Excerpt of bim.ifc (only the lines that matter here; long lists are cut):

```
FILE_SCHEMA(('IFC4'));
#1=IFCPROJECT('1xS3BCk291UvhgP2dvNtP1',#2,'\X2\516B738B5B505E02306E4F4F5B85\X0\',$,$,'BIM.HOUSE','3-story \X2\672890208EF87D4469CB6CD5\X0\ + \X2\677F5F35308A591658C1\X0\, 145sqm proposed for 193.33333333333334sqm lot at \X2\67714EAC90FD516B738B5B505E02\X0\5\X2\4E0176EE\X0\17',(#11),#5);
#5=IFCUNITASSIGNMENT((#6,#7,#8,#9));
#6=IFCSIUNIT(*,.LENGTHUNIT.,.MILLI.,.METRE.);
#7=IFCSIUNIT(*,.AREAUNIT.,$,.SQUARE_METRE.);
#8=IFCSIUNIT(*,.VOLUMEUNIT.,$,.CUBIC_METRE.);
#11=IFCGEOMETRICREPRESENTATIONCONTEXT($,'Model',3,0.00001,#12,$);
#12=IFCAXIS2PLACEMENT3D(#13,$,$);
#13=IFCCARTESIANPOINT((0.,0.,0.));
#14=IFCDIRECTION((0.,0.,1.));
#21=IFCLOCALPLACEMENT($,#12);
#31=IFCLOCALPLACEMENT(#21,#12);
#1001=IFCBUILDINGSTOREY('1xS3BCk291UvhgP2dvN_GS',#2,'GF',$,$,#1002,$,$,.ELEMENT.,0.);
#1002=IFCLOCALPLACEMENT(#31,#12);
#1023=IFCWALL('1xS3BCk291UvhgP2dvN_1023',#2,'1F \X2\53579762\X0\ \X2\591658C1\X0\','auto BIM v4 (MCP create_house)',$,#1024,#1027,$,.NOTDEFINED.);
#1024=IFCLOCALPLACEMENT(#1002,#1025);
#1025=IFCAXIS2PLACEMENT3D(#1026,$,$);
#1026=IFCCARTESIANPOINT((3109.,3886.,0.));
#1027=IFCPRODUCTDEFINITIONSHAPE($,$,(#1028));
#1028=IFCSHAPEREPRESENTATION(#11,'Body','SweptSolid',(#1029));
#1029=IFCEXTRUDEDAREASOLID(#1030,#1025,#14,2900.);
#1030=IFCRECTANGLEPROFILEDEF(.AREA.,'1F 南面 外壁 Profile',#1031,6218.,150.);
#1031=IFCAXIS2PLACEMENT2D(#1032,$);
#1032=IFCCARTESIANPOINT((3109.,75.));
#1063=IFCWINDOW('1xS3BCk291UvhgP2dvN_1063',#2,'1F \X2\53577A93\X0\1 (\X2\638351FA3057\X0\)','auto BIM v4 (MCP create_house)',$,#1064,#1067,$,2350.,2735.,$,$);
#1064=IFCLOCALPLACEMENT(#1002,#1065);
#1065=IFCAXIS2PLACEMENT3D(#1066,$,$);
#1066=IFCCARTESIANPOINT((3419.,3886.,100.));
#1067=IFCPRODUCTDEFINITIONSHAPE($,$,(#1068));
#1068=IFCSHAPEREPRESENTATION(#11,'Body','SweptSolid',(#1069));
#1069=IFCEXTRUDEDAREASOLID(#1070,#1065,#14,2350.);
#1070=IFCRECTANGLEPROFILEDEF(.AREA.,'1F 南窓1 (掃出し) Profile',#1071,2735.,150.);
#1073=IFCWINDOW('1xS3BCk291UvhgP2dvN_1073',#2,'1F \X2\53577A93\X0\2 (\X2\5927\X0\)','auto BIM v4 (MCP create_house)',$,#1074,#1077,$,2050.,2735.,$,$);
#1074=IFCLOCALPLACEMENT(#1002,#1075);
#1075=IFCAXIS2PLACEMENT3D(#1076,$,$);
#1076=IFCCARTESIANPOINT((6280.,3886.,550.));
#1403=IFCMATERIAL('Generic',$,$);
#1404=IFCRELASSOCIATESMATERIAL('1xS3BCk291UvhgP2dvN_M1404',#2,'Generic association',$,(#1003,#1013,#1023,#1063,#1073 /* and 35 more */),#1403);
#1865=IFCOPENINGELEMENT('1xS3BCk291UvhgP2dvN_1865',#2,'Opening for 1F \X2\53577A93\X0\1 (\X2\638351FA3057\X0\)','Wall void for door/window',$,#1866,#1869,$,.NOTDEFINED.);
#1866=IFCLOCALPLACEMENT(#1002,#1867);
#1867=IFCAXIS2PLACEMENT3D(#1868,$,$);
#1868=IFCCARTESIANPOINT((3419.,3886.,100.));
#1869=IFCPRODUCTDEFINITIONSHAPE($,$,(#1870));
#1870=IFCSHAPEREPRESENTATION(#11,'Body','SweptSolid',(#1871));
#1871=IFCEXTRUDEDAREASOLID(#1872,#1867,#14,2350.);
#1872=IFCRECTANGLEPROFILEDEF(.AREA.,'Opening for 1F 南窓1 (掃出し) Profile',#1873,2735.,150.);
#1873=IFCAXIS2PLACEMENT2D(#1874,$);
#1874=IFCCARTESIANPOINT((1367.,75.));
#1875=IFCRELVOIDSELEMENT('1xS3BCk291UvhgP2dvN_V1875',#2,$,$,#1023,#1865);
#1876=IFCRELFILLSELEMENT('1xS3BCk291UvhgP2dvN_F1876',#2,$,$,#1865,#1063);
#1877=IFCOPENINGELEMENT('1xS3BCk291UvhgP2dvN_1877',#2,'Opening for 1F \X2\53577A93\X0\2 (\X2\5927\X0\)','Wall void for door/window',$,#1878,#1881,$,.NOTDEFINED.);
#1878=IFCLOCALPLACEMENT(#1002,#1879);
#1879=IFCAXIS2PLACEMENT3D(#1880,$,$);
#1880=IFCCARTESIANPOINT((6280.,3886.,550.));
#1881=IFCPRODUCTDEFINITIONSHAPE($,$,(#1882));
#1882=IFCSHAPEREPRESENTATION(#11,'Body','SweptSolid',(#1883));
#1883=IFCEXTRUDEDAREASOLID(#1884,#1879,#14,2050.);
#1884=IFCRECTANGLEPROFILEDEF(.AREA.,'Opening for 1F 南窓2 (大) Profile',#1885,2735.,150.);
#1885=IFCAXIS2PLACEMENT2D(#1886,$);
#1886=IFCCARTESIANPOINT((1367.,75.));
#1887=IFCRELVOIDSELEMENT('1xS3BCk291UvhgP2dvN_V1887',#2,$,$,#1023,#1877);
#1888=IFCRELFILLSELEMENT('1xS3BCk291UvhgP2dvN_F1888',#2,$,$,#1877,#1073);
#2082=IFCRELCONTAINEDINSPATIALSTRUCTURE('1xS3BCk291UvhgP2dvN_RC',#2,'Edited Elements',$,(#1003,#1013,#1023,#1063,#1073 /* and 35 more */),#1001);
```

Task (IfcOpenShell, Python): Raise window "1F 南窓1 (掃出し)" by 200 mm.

```python
import numpy as np
import ifcopenshell
import ifcopenshell.api.geometry
import ifcopenshell.util.placement
import ifcopenshell.util.unit

model = ifcopenshell.open("bim.ifc")
unit_scale = ifcopenshell.util.unit.calculate_unit_scale(model)

window = model.by_guid("1xS3BCk291UvhgP2dvN_1063")
opening = window.FillsVoids[0].RelatingOpeningElement
dz = 200.0

shift = np.array([0.0, 0.0, dz])
# The window is not placed relative to its opening, so move both.
for product in (opening, window):
    matrix = ifcopenshell.util.placement.get_local_placement(product.ObjectPlacement)
    matrix[:3, 3] += shift
    ifcopenshell.api.geometry.edit_object_placement(model, product=product, matrix=matrix, is_si=False)

print(f"moved by {dz * unit_scale:+.3f} m")

model.write("bim-out.ifc")
```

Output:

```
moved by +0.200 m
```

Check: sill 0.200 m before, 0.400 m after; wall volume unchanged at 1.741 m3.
